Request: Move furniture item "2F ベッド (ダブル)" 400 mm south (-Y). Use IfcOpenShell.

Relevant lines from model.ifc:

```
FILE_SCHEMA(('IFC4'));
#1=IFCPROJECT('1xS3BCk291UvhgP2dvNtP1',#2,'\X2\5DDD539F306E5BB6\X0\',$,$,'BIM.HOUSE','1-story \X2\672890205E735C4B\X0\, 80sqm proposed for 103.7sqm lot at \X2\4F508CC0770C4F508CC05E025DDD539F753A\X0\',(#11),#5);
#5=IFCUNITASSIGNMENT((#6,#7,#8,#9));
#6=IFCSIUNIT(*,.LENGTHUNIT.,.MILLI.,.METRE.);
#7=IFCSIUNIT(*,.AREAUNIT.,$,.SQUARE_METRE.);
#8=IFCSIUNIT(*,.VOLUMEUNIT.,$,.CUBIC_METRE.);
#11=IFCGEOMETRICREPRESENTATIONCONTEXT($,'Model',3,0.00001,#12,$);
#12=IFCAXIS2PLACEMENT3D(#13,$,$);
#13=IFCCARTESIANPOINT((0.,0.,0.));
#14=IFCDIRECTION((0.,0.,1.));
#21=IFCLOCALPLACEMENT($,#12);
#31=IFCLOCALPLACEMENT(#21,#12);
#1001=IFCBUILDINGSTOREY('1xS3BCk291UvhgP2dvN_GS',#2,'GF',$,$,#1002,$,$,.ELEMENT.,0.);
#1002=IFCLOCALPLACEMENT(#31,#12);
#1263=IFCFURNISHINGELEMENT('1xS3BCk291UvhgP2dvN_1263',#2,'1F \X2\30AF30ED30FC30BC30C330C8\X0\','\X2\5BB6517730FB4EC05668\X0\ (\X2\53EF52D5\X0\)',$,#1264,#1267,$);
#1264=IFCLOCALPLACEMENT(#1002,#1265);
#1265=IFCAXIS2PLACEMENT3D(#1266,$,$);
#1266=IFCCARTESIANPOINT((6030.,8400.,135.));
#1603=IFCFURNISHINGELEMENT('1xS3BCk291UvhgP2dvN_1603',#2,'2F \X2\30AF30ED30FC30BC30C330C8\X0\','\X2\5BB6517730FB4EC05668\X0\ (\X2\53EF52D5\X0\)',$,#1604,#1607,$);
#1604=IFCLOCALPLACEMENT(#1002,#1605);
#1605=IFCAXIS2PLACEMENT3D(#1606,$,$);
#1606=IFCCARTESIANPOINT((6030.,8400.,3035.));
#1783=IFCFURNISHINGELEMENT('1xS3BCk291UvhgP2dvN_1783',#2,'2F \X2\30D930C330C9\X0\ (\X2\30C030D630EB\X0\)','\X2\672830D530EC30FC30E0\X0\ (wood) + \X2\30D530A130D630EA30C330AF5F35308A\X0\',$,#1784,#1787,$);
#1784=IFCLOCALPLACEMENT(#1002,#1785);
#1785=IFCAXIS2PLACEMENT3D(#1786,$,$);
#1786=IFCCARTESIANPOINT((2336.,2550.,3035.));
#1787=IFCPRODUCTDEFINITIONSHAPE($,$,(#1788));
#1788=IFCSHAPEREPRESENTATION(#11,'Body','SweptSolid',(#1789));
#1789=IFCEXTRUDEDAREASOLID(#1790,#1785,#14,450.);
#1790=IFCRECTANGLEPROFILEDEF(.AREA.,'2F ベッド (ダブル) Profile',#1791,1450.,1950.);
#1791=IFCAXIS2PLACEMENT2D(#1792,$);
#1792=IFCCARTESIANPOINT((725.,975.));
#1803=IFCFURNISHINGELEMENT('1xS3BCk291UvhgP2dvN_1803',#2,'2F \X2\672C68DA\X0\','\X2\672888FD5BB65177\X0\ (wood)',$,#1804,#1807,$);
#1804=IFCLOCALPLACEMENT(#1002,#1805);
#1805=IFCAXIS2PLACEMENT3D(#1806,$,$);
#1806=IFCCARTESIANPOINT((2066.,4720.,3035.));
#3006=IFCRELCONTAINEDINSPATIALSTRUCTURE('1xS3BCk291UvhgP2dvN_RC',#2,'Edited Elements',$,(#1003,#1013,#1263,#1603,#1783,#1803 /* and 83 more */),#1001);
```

```python
import ifcopenshell
import ifcopenshell.api.geometry
import ifcopenshell.util.placement
import ifcopenshell.util.unit

model = ifcopenshell.open("model.ifc")
unit_scale = ifcopenshell.util.unit.calculate_unit_scale(model)

item = model.by_id(1783)
matrix = ifcopenshell.util.placement.get_local_placement(item.ObjectPlacement)
matrix[1, 3] -= 0.4 / unit_scale
ifcopenshell.api.geometry.edit_object_placement(model, product=item, matrix=matrix, is_si=False)

print(ifcopenshell.util.placement.get_local_placement(item.ObjectPlacement).round(3) + 0.0)

model.write("model_updated.ifc")
```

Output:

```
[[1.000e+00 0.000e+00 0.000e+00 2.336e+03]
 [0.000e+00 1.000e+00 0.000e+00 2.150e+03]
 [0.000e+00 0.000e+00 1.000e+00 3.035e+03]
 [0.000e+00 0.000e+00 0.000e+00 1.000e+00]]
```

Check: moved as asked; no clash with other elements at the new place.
